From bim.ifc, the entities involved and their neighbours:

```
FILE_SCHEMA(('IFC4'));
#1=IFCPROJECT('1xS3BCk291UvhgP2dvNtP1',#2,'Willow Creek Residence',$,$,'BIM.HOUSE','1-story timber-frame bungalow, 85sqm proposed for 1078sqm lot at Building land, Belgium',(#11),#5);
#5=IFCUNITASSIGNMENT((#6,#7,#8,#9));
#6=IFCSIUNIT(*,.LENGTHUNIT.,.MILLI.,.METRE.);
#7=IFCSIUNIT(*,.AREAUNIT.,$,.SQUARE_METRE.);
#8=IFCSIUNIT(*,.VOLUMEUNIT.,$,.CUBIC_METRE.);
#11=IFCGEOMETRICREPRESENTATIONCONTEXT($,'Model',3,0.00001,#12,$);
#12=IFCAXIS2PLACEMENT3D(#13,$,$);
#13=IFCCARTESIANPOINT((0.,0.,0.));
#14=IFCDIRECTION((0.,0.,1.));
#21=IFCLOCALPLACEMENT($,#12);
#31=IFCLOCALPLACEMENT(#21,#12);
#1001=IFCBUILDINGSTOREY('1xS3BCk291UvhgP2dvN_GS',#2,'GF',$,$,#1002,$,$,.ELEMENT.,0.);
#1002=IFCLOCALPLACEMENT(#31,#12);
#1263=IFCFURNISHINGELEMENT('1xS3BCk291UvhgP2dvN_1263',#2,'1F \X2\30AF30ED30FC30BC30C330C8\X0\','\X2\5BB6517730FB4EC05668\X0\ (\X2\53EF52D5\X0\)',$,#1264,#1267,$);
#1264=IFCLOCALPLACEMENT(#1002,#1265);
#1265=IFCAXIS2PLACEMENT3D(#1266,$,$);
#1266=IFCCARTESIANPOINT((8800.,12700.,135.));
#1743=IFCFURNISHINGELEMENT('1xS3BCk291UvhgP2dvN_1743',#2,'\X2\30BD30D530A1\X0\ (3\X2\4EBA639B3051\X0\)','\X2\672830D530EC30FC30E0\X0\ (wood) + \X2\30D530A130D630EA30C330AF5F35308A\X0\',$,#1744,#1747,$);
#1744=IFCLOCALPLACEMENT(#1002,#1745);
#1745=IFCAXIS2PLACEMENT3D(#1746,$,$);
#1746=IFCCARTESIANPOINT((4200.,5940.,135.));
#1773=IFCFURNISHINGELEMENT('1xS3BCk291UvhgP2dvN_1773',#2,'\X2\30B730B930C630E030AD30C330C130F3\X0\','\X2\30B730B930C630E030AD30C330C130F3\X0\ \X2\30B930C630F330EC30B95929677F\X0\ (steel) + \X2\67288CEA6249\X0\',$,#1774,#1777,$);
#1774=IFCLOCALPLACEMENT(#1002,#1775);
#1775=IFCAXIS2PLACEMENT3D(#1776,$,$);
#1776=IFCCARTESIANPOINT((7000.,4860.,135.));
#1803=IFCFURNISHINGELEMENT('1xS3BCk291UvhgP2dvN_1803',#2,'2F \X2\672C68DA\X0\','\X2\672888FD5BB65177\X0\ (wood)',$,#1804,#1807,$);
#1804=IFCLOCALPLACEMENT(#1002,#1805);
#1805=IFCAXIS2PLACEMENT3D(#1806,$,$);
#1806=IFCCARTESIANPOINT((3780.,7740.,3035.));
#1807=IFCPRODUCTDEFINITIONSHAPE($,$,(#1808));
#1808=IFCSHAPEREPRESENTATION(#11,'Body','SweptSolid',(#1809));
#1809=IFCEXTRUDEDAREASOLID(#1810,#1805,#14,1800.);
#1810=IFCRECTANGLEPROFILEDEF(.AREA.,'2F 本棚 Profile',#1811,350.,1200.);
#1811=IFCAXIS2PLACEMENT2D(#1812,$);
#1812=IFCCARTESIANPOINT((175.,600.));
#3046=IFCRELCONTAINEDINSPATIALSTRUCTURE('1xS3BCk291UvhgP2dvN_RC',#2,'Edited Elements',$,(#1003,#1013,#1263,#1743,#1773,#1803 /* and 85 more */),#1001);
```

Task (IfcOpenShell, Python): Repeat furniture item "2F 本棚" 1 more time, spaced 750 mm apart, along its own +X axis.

```python
import ifcopenshell
import ifcopenshell.api.geometry
import ifcopenshell.api.root
import ifcopenshell.util.element
import ifcopenshell.util.placement

model = ifcopenshell.open("bim.ifc")


def reuse_history(source, copy):
    """copy_class also copies each property set's owner history, people and application; keep the originals."""
    for rel in copy.IsDefinedBy:
        if rel.is_a("IfcRelDefinesByProperties") and (history := rel.RelatingPropertyDefinition.OwnerHistory):
            rel.RelatingPropertyDefinition.OwnerHistory = source.OwnerHistory
            ifcopenshell.util.element.remove_deep2(model, history)


source = model.by_guid("1xS3BCk291UvhgP2dvN_1803")
base = ifcopenshell.util.placement.get_local_placement(source.ObjectPlacement)
step = base[:3, 0] * 750.0

for i in range(1, 2):
    copy = ifcopenshell.api.root.copy_class(model, product=source)
    copy.Representation = ifcopenshell.util.element.copy_deep(
        model, source.Representation, exclude=["IfcGeometricRepresentationContext", "IfcRepresentationMap"]
    )
    reuse_history(source, copy)
    matrix = base.copy()
    matrix[:3, 3] += i * step
    print("added at", matrix[:3, 3].round(3) + 0.0)
    ifcopenshell.api.geometry.edit_object_placement(model, product=copy, matrix=matrix, is_si=False)

model.write("bim_rev.ifc")
```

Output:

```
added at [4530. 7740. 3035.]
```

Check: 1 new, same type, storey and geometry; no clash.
